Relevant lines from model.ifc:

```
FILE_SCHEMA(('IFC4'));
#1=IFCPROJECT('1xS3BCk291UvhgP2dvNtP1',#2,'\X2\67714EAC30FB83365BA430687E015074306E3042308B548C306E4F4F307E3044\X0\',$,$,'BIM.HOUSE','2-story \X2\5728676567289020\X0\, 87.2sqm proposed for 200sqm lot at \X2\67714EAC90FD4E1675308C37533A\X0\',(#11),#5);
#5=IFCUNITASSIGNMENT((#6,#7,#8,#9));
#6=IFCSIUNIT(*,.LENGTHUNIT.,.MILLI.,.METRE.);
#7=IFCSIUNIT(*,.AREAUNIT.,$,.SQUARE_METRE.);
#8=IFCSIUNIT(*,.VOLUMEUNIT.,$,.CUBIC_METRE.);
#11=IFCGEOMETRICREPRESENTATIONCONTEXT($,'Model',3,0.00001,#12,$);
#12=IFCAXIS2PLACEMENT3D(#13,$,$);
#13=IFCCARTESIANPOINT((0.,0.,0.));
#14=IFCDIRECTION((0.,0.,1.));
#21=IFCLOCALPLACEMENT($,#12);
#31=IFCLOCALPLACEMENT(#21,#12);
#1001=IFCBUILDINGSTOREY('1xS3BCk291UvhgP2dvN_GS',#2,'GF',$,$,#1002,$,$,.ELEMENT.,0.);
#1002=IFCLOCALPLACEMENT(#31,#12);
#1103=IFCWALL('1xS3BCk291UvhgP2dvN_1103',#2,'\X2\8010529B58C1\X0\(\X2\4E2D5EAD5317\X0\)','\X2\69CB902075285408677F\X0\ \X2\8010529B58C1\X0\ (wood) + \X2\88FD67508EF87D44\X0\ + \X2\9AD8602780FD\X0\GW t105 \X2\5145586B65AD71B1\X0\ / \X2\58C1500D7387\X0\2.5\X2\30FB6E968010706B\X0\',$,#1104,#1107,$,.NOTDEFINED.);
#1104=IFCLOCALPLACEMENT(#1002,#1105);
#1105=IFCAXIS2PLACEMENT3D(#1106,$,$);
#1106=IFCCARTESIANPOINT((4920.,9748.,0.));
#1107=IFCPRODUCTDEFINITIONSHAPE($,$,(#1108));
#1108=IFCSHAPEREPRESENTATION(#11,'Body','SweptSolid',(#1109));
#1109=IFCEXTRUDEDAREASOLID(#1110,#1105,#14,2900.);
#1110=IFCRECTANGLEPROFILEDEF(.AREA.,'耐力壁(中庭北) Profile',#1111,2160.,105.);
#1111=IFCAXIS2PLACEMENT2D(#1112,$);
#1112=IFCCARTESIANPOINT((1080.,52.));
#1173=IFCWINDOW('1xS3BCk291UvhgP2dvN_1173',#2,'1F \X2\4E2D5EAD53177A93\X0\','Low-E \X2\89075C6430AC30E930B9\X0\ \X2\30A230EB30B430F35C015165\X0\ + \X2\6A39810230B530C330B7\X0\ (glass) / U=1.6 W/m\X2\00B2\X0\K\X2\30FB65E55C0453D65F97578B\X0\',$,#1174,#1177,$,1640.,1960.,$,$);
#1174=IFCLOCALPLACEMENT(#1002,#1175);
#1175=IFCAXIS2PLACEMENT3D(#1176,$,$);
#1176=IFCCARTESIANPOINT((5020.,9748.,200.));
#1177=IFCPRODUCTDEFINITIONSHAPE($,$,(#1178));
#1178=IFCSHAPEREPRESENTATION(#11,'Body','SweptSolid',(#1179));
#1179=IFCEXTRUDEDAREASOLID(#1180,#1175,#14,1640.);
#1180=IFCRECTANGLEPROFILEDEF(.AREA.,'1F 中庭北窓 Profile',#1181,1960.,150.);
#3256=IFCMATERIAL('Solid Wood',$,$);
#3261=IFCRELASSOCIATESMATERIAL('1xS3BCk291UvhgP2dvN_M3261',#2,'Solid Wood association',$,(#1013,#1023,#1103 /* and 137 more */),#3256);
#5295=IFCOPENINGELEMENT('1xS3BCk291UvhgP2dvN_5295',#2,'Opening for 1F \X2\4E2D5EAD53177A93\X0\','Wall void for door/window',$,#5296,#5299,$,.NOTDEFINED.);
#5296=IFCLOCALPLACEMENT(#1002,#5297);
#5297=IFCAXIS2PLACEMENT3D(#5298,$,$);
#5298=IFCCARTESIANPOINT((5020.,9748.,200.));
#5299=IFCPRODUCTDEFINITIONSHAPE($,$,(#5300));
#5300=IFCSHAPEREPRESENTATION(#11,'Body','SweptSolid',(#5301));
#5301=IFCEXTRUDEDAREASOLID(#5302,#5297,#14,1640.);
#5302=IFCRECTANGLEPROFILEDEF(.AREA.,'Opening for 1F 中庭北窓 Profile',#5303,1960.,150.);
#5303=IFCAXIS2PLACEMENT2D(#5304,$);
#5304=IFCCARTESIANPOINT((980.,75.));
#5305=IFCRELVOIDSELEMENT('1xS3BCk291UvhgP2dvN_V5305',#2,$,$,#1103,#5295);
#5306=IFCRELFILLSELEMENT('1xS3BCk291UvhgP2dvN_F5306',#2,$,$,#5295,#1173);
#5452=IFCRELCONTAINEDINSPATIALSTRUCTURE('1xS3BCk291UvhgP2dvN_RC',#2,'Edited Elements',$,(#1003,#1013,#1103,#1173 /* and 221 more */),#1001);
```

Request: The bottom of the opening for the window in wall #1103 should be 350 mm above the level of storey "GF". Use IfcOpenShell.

```python
import numpy as np
import ifcopenshell
import ifcopenshell.api.geometry
import ifcopenshell.geom
import ifcopenshell.util.element
import ifcopenshell.util.placement
import ifcopenshell.util.shape
import ifcopenshell.util.unit

model = ifcopenshell.open("model.ifc")
unit_scale = ifcopenshell.util.unit.calculate_unit_scale(model)

window = model.by_guid("1xS3BCk291UvhgP2dvN_1173")
opening = window.FillsVoids[0].RelatingOpeningElement
storey = ifcopenshell.util.element.get_container(window, ifc_class="IfcBuildingStorey")
level = ifcopenshell.util.placement.get_local_placement(storey.ObjectPlacement)[2, 3]

# The opening's origin need not be at the sill, so measure its lowest point.
shape = ifcopenshell.geom.create_shape(ifcopenshell.geom.settings(), opening)
bottom = ifcopenshell.util.shape.get_shape_bottom_elevation(shape, shape.geometry) / unit_scale
dz = level + 0.35 / unit_scale - bottom

shift = np.array([0.0, 0.0, dz])
# The window is not placed relative to its opening, so move both.
for product in (opening, window):
    matrix = ifcopenshell.util.placement.get_local_placement(product.ObjectPlacement)
    matrix[:3, 3] += shift
    ifcopenshell.api.geometry.edit_object_placement(model, product=product, matrix=matrix, is_si=False)

print(f"moved by {dz * unit_scale:+.3f} m")

model.write("model_v2.ifc")
```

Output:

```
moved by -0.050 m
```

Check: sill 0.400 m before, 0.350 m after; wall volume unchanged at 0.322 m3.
